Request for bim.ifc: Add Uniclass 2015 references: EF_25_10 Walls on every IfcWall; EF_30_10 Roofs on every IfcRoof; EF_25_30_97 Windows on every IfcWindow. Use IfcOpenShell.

First a look at what the model holds.

```python
import ifcopenshell

model = ifcopenshell.open("bim.ifc")
print(model.schema)
print("classifications:", [c.Name for c in model.by_type("IfcClassification")])
for ifc_class in ("IfcDoor", "IfcRoof", "IfcStair", "IfcWall", "IfcWindow"):
    print(ifc_class, len(model.by_type(ifc_class)))
```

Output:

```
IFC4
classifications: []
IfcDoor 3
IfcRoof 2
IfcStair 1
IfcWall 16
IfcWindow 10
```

```python
import ifcopenshell
import ifcopenshell.api.classification

model = ifcopenshell.open("bim.ifc")

system = ifcopenshell.api.classification.add_classification(model, classification="Uniclass 2015")

codes = {
    "IfcWall": ("EF_25_10", "Walls"),
    "IfcRoof": ("EF_30_10", "Roofs"),
    "IfcWindow": ("EF_25_30_97", "Windows"),
}
for ifc_class, (code, name) in codes.items():
    products = model.by_type(ifc_class)
    ifcopenshell.api.classification.add_reference(
        model, products=products, classification=system, identification=code, name=name
    )
    print(code, len(products))

model.write("bim-out.ifc")
```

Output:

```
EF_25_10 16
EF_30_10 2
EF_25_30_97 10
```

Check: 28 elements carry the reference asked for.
